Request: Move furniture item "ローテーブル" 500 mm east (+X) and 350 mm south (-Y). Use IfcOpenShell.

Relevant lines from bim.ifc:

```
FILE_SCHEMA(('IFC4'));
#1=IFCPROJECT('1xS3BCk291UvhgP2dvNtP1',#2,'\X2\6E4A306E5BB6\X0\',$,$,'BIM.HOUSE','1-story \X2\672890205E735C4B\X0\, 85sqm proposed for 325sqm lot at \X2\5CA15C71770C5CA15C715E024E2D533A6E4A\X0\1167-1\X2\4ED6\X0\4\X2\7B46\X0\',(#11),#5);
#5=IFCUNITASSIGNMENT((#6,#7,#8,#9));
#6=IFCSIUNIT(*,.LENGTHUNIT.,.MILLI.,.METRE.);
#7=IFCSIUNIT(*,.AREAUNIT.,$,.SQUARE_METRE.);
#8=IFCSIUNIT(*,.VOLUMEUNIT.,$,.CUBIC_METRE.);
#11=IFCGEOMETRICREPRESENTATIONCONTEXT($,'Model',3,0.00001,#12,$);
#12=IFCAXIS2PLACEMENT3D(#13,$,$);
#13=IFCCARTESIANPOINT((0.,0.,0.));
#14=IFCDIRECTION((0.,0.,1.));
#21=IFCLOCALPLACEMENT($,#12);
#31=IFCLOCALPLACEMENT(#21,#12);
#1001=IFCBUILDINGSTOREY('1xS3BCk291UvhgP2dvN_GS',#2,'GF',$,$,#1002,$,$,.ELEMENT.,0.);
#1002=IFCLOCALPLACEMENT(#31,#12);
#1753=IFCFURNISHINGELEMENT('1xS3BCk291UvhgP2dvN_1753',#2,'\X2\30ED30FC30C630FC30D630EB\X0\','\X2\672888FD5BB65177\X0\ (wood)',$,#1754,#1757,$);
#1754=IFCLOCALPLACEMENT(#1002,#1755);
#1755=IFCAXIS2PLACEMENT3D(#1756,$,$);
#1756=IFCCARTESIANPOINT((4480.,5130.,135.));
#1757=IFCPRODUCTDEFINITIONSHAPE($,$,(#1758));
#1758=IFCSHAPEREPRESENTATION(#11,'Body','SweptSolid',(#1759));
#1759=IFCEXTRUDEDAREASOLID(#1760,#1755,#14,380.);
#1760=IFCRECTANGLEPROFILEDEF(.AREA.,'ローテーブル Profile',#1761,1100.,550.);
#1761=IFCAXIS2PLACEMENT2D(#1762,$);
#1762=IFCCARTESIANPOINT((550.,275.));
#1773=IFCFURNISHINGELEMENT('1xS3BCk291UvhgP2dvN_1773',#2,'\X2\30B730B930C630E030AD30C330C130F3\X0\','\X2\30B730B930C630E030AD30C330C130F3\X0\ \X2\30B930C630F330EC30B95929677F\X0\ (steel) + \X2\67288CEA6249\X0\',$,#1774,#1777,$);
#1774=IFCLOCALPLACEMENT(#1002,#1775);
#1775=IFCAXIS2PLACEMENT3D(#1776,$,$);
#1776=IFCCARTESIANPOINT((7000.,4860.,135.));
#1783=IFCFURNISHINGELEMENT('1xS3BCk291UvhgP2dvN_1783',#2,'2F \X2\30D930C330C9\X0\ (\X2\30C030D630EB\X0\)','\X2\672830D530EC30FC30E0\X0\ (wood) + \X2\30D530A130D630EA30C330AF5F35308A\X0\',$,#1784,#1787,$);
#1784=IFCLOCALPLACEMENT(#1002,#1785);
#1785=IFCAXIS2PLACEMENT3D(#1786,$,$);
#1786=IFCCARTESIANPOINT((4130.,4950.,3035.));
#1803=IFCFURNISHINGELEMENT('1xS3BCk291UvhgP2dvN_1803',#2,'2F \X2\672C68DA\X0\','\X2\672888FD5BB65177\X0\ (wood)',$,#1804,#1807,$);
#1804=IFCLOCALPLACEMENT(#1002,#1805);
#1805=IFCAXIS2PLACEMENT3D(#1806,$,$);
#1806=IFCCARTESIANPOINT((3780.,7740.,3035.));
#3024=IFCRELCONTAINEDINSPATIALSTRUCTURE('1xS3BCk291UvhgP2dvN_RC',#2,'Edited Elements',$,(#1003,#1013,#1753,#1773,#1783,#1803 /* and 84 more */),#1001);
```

```python
import ifcopenshell
import ifcopenshell.api.geometry
import ifcopenshell.util.placement

model = ifcopenshell.open("bim.ifc")

item = model.by_id(1753)
matrix = ifcopenshell.util.placement.get_local_placement(item.ObjectPlacement)
matrix[0, 3] += 500.0
matrix[1, 3] -= 350.0
ifcopenshell.api.geometry.edit_object_placement(model, product=item, matrix=matrix, is_si=False)

print(ifcopenshell.util.placement.get_local_placement(item.ObjectPlacement).round(3) + 0.0)

model.write("bim_rev.ifc")
```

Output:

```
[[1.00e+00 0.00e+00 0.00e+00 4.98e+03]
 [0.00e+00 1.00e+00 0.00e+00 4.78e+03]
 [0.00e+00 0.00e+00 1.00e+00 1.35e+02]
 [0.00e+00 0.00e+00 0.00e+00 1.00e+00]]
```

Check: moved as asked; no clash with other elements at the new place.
